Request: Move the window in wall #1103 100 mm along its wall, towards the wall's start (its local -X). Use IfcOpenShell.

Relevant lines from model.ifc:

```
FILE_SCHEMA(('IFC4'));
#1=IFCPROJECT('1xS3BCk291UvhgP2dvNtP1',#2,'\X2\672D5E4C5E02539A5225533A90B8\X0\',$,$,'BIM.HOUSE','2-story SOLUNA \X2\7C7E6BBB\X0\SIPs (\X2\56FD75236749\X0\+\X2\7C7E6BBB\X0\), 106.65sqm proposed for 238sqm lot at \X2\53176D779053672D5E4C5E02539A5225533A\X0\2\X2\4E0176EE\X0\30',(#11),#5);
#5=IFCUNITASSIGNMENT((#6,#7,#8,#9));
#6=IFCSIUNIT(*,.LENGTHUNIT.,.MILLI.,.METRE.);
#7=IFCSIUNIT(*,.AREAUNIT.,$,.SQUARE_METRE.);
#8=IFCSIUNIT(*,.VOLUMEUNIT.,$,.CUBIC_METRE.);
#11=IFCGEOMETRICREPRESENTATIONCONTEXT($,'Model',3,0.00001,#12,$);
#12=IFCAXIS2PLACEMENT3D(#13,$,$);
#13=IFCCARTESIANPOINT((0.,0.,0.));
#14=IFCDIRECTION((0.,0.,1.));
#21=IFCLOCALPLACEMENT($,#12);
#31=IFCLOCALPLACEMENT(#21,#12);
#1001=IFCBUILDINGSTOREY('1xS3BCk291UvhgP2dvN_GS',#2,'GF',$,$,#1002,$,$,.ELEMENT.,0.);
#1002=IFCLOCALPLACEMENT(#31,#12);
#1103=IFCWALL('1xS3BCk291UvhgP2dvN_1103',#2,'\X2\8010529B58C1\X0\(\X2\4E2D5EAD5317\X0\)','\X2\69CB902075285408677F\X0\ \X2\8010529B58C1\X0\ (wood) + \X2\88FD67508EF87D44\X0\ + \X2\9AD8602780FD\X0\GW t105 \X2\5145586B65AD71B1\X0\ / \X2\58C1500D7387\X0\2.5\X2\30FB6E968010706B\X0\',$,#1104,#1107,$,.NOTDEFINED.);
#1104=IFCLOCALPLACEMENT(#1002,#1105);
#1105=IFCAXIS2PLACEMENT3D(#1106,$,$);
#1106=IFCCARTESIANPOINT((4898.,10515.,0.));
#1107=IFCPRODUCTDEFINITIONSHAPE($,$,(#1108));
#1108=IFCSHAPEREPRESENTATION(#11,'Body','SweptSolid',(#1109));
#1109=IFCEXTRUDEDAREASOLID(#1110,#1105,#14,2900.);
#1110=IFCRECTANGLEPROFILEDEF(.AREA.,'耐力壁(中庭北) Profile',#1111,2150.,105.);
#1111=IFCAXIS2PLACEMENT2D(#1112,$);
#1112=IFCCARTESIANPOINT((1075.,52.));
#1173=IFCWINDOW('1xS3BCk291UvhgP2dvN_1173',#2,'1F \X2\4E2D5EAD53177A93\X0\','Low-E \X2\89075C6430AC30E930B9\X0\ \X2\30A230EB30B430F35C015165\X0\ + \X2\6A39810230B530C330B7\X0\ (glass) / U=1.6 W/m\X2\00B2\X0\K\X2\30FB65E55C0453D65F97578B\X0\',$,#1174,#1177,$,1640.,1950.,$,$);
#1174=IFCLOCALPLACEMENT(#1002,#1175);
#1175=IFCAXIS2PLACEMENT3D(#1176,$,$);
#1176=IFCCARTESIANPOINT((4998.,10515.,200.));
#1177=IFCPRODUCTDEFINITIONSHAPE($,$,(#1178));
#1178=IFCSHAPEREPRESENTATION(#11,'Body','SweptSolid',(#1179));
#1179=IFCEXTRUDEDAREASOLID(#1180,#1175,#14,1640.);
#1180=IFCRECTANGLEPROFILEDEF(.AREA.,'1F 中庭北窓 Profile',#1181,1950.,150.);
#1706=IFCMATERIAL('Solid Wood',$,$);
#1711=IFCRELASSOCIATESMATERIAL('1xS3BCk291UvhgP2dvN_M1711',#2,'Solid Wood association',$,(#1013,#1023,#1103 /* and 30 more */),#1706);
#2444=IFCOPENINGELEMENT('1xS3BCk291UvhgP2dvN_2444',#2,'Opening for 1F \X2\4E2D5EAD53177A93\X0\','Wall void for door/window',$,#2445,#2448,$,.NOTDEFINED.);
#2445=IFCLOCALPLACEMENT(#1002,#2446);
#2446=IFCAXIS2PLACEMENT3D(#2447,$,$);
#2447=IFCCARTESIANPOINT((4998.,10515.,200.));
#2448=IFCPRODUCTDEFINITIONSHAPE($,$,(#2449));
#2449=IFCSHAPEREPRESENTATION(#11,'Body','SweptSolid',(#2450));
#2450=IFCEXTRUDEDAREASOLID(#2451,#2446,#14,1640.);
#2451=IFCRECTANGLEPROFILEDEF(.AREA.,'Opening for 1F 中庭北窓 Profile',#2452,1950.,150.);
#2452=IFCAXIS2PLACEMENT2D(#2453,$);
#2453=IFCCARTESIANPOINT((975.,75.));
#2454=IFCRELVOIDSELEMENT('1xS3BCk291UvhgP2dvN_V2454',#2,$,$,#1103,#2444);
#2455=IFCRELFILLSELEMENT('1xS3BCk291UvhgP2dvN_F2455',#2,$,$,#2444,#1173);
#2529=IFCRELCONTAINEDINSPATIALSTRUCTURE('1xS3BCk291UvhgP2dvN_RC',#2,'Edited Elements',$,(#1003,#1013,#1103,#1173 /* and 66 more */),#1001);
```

```python
import ifcopenshell
import ifcopenshell.api.geometry
import ifcopenshell.util.placement
import ifcopenshell.util.unit

model = ifcopenshell.open("model.ifc")
unit_scale = ifcopenshell.util.unit.calculate_unit_scale(model)

window = model.by_guid("1xS3BCk291UvhgP2dvN_1173")
opening = window.FillsVoids[0].RelatingOpeningElement
wall = opening.VoidsElements[0].RelatingBuildingElement

wall_matrix = ifcopenshell.util.placement.get_local_placement(wall.ObjectPlacement)
shift = wall_matrix[:3, 0] * -0.1 / unit_scale
before = ifcopenshell.util.placement.get_local_placement(window.ObjectPlacement)[:3, 3].copy()

# The window is not placed relative to its opening, so move both.
for product in (opening, window):
    matrix = ifcopenshell.util.placement.get_local_placement(product.ObjectPlacement)
    matrix[:3, 3] += shift
    ifcopenshell.api.geometry.edit_object_placement(model, product=product, matrix=matrix, is_si=False)

after = ifcopenshell.util.placement.get_local_placement(window.ObjectPlacement)[:3, 3]
print("window moved by", (after - before).round(3) + 0.0)

model.write("model_rev.ifc")
```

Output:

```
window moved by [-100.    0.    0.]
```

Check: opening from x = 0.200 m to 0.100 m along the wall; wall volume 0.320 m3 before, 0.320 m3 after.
